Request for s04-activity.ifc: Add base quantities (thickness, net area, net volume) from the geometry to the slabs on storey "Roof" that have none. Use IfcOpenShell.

First a look at what the model holds.

```python
import ifcopenshell
import ifcopenshell.util.element
import ifcopenshell.util.unit

model = ifcopenshell.open("s04-activity.ifc")
print(model.schema)
for unit_type in ("LENGTHUNIT", "AREAUNIT", "VOLUMEUNIT"):
    print(unit_type, ifcopenshell.util.unit.calculate_unit_scale(model, unit_type))
storey = next(s for s in model.by_type("IfcBuildingStorey") if s.Name == "Roof")
slabs = [e for e in ifcopenshell.util.element.get_decomposition(storey) if e.is_a("IfcSlab")]
for e in sorted(slabs, key=lambda e: e.id()):
    print(e.id(), e.is_a(), e.Name, list(ifcopenshell.util.element.get_psets(e, qtos_only=True)), sep=" | ")
```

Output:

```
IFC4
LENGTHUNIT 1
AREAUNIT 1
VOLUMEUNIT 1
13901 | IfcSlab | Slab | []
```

```python
import ifcopenshell
import ifcopenshell.api.pset
import ifcopenshell.geom
import ifcopenshell.util.element
import ifcopenshell.util.shape
import ifcopenshell.util.unit

model = ifcopenshell.open("s04-activity.ifc")
unit_scale = ifcopenshell.util.unit.calculate_unit_scale(model)
area_scale = ifcopenshell.util.unit.calculate_unit_scale(model, "AREAUNIT")
volume_scale = ifcopenshell.util.unit.calculate_unit_scale(model, "VOLUMEUNIT")
settings = ifcopenshell.geom.settings()

storey = next(s for s in model.by_type("IfcBuildingStorey") if s.Name == "Roof")
slabs = [e for e in ifcopenshell.util.element.get_decomposition(storey) if e.is_a("IfcSlab")]

for e in sorted(slabs, key=lambda e: e.id()):
    if ifcopenshell.util.element.get_psets(e, qtos_only=True, should_inherit=False):
        continue
    # Geometry comes back in metres, in the element's own axes.
    shape = ifcopenshell.geom.create_shape(settings, e)
    values = {
        "Width": ifcopenshell.util.shape.get_z(shape.geometry) / unit_scale,
        "NetArea": ifcopenshell.util.shape.get_footprint_area(shape.geometry) / area_scale,
        "NetVolume": ifcopenshell.util.shape.get_volume(shape.geometry) / volume_scale,
    }
    qto = ifcopenshell.api.pset.add_qto(model, product=e, name="Qto_SlabBaseQuantities")
    ifcopenshell.api.pset.edit_qto(model, qto=qto, properties=values)
    print(e.id(), {k: round(v, 3) for k, v in values.items()})

model.write("s04-activity_v2.ifc")
```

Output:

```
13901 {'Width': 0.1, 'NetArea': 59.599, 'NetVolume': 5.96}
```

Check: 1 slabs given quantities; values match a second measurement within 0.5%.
